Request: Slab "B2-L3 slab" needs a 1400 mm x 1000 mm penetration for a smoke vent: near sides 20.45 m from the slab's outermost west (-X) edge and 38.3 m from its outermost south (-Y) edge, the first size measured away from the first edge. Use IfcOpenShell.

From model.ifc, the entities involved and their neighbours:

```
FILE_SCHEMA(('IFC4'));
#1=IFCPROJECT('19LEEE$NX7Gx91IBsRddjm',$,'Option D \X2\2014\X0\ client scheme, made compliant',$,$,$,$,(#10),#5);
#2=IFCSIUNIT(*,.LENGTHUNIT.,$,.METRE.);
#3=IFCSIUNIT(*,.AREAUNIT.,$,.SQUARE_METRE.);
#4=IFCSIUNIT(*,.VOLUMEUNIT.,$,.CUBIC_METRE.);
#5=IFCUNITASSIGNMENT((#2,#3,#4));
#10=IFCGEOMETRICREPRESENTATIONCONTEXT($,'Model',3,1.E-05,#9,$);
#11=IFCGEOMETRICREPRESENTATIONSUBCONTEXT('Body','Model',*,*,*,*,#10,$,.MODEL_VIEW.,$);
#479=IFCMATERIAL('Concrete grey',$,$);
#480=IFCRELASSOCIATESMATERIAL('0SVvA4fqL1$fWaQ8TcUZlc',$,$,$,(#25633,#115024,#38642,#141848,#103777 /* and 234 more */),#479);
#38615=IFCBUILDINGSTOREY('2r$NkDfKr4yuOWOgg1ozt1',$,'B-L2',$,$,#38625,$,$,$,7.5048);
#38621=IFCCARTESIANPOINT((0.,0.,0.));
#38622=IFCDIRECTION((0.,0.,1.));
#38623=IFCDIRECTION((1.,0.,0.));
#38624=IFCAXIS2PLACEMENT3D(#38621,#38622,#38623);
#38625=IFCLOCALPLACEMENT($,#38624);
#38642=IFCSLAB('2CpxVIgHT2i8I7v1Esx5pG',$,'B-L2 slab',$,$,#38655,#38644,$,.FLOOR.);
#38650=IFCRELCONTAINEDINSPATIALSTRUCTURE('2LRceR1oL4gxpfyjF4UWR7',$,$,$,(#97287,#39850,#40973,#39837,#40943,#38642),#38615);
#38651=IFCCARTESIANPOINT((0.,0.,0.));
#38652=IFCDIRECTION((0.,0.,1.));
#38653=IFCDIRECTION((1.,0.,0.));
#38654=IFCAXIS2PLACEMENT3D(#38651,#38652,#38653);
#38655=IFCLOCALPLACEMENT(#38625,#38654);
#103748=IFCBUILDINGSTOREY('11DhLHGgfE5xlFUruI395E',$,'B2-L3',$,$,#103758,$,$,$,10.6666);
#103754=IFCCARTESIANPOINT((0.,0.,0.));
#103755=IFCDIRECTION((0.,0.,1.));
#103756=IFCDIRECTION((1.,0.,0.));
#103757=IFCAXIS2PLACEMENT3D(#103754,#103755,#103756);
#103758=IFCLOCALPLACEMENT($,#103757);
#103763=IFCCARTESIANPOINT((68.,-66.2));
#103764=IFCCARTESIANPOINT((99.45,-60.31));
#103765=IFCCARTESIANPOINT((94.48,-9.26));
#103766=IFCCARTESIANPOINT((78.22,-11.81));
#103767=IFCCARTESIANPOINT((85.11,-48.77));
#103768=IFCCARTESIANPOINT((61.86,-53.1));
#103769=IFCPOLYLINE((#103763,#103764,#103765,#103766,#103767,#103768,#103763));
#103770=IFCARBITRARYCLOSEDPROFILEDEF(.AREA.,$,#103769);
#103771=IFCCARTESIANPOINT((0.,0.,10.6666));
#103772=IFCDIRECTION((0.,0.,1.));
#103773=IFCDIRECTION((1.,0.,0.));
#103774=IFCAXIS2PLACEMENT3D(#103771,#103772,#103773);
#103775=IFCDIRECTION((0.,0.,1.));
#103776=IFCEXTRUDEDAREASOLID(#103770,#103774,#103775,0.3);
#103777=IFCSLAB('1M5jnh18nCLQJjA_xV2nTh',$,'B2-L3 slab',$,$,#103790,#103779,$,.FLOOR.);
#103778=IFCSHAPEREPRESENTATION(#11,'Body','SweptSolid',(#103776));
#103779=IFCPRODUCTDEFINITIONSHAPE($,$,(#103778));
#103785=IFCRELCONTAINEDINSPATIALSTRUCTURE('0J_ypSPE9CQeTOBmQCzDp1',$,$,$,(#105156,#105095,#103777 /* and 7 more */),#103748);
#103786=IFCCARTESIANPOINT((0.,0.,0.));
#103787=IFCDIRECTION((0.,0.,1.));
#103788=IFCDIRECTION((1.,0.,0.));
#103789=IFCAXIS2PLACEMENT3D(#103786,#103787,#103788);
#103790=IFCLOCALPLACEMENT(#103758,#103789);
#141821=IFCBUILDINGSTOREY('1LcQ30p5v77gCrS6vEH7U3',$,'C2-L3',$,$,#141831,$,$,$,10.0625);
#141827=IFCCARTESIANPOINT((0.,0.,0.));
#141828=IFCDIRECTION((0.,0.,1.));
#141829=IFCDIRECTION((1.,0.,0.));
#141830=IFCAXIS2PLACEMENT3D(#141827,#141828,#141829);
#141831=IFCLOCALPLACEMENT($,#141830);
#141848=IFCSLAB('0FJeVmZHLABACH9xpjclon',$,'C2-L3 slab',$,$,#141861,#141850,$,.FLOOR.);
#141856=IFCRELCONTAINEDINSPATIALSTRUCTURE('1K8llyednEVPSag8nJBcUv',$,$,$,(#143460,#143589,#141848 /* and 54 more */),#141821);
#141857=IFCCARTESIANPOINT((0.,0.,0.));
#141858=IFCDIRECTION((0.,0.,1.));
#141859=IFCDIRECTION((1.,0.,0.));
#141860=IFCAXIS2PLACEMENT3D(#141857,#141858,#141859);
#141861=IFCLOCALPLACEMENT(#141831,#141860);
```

```python
import numpy as np
import ifcopenshell
import ifcopenshell.api.feature
import ifcopenshell.api.geometry
import ifcopenshell.api.root
import ifcopenshell.geom
import ifcopenshell.util.placement
import ifcopenshell.util.representation
import ifcopenshell.util.shape
import ifcopenshell.util.unit

model = ifcopenshell.open("model.ifc")
unit_scale = ifcopenshell.util.unit.calculate_unit_scale(model)
settings = ifcopenshell.geom.settings()


def volume(element):
    """Net volume in cubic metres, openings subtracted."""
    shape = ifcopenshell.geom.create_shape(settings, element)
    return ifcopenshell.util.shape.get_volume(shape.geometry)


slab = model.by_guid("1M5jnh18nCLQJjA_xV2nTh")
before = volume(slab)

# Extent in the slab's own axes, in metres. The edges named are its -X and -Y sides.
slab_shape = ifcopenshell.geom.create_shape(settings, slab)
vertices = ifcopenshell.util.shape.get_vertices(slab_shape.geometry)
x_min, y_min, bottom = vertices.min(axis=0)
top = vertices[:, 2].max()

opening = ifcopenshell.api.root.create_entity(model, ifc_class="IfcOpeningElement", name="Smoke vent opening", predefined_type="OPENING")
context = ifcopenshell.util.representation.get_context(model, "Model", "Body", "MODEL_VIEW")
width, depth = 1.4, 1
outline = [(0.0, 0.0), (width, 0.0), (width, depth), (0.0, depth), (0.0, 0.0)]
# Overshoot both faces by 50 mm so the cut is clean.
shape = ifcopenshell.api.geometry.add_slab_representation(
    model, context=context, depth=top - bottom + 0.1, polyline=outline
)
ifcopenshell.api.geometry.assign_representation(model, product=opening, representation=shape)

matrix = ifcopenshell.util.placement.get_local_placement(slab.ObjectPlacement)
matrix[:, 3] = matrix @ np.append(np.array([x_min + 20.45, y_min + 38.3, bottom - 0.05]) / unit_scale, 1.0)
ifcopenshell.api.geometry.edit_object_placement(model, product=opening, matrix=matrix, is_si=False)
ifcopenshell.api.feature.add_feature(model, feature=opening, element=slab)

after = volume(slab)

print(f"slab volume {before:.3f} -> {after:.3f} m3")

model.write("model-out.ifc")
```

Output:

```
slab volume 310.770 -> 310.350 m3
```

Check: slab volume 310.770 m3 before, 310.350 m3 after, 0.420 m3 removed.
